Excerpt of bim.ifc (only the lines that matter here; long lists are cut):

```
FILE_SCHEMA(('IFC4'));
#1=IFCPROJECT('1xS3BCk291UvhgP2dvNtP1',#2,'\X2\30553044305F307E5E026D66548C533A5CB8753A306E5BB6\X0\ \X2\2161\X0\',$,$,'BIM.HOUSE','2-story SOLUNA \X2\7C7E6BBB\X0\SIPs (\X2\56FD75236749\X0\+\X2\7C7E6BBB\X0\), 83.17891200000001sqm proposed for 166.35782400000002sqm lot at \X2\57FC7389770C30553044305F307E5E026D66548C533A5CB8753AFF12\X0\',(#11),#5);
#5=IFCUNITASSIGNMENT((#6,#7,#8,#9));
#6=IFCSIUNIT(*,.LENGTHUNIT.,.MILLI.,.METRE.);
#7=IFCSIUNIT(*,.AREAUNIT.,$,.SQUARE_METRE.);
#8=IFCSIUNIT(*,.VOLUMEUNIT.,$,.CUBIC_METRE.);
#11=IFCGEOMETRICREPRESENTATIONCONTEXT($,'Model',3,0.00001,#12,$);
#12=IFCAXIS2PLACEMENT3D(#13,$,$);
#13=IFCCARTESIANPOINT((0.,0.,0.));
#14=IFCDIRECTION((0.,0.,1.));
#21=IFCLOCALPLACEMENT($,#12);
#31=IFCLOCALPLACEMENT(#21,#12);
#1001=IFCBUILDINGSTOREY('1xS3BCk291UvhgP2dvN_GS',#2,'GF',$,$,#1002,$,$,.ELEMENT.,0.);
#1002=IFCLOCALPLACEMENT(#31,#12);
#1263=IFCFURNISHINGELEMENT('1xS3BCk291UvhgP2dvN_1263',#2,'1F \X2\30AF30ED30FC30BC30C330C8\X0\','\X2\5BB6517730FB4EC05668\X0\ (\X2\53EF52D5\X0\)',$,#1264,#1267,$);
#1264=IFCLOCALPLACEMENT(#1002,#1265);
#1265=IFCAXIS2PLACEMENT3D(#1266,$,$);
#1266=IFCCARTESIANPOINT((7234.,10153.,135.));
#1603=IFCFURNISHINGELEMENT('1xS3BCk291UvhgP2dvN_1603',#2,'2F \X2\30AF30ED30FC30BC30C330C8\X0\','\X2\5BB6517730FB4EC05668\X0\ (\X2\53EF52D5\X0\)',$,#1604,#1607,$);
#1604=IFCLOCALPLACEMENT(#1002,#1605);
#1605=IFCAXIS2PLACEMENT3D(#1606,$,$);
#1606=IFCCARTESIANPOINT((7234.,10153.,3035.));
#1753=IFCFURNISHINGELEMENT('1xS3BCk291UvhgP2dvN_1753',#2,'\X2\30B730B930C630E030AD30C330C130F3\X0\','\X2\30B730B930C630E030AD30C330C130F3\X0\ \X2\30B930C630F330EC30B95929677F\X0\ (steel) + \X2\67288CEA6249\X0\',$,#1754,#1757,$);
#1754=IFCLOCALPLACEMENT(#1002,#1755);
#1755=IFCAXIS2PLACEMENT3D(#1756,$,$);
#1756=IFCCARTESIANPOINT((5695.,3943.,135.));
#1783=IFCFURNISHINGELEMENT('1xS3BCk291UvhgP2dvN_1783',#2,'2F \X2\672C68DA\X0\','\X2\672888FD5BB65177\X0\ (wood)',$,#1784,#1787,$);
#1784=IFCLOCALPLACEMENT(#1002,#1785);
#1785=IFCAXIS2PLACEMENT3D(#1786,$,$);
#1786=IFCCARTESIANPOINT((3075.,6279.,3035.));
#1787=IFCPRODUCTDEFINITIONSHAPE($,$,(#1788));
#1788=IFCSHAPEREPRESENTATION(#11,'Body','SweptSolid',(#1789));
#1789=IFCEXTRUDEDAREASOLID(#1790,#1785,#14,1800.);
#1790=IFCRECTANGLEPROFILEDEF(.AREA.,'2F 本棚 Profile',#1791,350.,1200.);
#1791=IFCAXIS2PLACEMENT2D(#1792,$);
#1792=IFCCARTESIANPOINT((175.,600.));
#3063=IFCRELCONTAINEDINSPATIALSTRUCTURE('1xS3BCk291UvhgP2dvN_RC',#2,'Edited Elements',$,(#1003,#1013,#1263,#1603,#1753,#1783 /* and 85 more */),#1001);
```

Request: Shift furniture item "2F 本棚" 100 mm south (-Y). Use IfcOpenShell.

```python
import ifcopenshell
import ifcopenshell.api.geometry
import ifcopenshell.util.placement
import ifcopenshell.util.unit

model = ifcopenshell.open("bim.ifc")
unit_scale = ifcopenshell.util.unit.calculate_unit_scale(model)

item = model.by_id(1783)
matrix = ifcopenshell.util.placement.get_local_placement(item.ObjectPlacement)
matrix[1, 3] -= 0.1 / unit_scale
ifcopenshell.api.geometry.edit_object_placement(model, product=item, matrix=matrix, is_si=False)

print(ifcopenshell.util.placement.get_local_placement(item.ObjectPlacement).round(3) + 0.0)

model.write("bim_v2.ifc")
```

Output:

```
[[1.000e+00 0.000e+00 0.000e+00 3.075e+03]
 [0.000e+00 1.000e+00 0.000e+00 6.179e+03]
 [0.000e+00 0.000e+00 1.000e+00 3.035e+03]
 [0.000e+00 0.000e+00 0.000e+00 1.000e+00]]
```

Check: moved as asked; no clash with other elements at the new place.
